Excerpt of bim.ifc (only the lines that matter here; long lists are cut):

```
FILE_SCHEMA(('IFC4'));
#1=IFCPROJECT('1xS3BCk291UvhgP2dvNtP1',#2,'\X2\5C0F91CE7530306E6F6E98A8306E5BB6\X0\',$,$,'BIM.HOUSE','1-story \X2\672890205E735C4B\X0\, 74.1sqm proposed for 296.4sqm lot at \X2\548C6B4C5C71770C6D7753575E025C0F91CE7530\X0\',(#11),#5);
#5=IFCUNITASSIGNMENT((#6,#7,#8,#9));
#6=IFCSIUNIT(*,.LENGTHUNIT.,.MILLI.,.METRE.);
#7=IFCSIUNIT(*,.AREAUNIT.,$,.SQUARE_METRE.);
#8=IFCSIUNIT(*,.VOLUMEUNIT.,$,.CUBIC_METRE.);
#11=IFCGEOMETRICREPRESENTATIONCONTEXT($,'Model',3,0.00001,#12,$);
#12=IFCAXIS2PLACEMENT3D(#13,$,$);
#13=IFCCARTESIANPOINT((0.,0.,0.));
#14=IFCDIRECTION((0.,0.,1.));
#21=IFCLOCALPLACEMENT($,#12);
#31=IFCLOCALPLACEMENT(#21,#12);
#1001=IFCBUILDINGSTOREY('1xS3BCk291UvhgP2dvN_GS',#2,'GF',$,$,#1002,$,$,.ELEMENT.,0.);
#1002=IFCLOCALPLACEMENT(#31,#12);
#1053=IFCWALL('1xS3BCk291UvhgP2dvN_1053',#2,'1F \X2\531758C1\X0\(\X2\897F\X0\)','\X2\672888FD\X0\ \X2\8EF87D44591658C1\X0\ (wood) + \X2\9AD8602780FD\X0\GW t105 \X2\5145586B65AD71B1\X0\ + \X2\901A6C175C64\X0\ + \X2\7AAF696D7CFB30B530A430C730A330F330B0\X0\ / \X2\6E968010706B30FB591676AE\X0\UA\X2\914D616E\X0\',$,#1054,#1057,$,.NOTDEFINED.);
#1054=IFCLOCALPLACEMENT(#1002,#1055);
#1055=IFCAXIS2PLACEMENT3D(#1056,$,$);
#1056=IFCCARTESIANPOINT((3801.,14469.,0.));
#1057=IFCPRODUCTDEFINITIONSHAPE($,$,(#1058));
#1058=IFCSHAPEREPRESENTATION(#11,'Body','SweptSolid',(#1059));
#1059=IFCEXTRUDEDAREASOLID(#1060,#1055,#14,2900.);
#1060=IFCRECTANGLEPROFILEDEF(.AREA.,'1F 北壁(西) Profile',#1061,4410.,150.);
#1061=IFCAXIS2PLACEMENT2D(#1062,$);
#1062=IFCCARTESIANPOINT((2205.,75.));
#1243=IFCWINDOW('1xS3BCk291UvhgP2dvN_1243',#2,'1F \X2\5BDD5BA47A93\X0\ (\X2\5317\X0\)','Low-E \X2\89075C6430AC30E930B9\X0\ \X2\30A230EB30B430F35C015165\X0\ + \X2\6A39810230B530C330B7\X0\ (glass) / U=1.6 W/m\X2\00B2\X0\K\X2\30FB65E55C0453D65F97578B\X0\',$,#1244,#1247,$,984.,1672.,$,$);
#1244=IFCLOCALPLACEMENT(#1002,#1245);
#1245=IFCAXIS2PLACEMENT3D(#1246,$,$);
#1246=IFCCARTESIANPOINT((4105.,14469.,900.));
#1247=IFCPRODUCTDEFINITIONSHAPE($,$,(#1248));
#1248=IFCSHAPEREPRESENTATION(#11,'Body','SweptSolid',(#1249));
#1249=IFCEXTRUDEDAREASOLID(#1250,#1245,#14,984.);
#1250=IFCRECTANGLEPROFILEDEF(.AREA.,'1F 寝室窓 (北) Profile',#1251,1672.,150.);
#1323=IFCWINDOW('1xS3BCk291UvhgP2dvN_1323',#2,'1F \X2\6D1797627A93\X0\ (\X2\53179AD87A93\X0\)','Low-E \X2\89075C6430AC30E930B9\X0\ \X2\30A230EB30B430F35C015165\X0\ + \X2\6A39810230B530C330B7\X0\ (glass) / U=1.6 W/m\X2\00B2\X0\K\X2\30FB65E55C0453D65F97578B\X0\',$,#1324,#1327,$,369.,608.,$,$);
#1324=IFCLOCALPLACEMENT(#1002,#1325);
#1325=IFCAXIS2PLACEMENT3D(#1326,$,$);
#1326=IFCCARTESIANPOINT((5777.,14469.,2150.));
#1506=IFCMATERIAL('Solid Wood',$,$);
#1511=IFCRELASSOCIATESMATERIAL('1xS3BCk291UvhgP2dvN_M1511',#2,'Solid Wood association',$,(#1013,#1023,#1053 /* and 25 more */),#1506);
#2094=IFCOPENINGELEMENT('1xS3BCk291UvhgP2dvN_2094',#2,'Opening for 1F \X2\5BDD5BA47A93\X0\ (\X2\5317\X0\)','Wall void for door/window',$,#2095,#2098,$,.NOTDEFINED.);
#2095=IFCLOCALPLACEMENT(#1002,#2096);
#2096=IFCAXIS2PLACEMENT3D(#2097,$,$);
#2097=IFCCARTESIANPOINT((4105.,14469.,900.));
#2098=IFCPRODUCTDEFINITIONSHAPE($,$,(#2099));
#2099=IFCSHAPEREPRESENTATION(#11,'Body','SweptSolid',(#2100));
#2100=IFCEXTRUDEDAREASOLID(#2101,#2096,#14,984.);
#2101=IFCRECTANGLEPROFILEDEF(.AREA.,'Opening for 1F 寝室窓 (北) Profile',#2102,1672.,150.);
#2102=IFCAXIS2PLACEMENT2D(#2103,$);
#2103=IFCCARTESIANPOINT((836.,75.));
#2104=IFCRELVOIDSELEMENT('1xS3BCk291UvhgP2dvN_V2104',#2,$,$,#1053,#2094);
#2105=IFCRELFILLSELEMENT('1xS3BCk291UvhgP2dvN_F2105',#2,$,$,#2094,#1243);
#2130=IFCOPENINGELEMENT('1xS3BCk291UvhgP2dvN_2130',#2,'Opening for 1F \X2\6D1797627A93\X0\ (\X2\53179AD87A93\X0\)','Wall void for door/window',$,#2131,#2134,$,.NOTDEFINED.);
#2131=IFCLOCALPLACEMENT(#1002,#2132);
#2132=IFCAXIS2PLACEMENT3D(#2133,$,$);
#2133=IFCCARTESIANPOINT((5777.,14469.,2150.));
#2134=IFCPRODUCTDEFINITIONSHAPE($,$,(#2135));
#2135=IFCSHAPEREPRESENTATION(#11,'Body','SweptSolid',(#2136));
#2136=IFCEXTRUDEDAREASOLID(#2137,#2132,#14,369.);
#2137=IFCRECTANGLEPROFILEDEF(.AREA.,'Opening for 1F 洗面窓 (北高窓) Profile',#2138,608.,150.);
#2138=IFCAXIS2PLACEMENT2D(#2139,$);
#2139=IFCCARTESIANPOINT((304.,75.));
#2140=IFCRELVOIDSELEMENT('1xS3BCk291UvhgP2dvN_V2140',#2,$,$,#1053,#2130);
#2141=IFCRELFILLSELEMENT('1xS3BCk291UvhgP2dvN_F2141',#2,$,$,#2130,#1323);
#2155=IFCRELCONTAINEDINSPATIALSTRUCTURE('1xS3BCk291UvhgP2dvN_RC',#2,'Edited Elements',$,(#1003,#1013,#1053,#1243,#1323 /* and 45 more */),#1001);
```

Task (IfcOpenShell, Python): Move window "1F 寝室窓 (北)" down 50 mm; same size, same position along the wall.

```python
import numpy as np
import ifcopenshell
import ifcopenshell.api.geometry
import ifcopenshell.util.placement
import ifcopenshell.util.unit

model = ifcopenshell.open("bim.ifc")
unit_scale = ifcopenshell.util.unit.calculate_unit_scale(model)

window = model.by_guid("1xS3BCk291UvhgP2dvN_1243")
opening = window.FillsVoids[0].RelatingOpeningElement
dz = -50.0

shift = np.array([0.0, 0.0, dz])
# The window is not placed relative to its opening, so move both.
for product in (opening, window):
    matrix = ifcopenshell.util.placement.get_local_placement(product.ObjectPlacement)
    matrix[:3, 3] += shift
    ifcopenshell.api.geometry.edit_object_placement(model, product=product, matrix=matrix, is_si=False)

print(f"moved by {dz * unit_scale:+.3f} m")

model.write("bim_edited.ifc")
```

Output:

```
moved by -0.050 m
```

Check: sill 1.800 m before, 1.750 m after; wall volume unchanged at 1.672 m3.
